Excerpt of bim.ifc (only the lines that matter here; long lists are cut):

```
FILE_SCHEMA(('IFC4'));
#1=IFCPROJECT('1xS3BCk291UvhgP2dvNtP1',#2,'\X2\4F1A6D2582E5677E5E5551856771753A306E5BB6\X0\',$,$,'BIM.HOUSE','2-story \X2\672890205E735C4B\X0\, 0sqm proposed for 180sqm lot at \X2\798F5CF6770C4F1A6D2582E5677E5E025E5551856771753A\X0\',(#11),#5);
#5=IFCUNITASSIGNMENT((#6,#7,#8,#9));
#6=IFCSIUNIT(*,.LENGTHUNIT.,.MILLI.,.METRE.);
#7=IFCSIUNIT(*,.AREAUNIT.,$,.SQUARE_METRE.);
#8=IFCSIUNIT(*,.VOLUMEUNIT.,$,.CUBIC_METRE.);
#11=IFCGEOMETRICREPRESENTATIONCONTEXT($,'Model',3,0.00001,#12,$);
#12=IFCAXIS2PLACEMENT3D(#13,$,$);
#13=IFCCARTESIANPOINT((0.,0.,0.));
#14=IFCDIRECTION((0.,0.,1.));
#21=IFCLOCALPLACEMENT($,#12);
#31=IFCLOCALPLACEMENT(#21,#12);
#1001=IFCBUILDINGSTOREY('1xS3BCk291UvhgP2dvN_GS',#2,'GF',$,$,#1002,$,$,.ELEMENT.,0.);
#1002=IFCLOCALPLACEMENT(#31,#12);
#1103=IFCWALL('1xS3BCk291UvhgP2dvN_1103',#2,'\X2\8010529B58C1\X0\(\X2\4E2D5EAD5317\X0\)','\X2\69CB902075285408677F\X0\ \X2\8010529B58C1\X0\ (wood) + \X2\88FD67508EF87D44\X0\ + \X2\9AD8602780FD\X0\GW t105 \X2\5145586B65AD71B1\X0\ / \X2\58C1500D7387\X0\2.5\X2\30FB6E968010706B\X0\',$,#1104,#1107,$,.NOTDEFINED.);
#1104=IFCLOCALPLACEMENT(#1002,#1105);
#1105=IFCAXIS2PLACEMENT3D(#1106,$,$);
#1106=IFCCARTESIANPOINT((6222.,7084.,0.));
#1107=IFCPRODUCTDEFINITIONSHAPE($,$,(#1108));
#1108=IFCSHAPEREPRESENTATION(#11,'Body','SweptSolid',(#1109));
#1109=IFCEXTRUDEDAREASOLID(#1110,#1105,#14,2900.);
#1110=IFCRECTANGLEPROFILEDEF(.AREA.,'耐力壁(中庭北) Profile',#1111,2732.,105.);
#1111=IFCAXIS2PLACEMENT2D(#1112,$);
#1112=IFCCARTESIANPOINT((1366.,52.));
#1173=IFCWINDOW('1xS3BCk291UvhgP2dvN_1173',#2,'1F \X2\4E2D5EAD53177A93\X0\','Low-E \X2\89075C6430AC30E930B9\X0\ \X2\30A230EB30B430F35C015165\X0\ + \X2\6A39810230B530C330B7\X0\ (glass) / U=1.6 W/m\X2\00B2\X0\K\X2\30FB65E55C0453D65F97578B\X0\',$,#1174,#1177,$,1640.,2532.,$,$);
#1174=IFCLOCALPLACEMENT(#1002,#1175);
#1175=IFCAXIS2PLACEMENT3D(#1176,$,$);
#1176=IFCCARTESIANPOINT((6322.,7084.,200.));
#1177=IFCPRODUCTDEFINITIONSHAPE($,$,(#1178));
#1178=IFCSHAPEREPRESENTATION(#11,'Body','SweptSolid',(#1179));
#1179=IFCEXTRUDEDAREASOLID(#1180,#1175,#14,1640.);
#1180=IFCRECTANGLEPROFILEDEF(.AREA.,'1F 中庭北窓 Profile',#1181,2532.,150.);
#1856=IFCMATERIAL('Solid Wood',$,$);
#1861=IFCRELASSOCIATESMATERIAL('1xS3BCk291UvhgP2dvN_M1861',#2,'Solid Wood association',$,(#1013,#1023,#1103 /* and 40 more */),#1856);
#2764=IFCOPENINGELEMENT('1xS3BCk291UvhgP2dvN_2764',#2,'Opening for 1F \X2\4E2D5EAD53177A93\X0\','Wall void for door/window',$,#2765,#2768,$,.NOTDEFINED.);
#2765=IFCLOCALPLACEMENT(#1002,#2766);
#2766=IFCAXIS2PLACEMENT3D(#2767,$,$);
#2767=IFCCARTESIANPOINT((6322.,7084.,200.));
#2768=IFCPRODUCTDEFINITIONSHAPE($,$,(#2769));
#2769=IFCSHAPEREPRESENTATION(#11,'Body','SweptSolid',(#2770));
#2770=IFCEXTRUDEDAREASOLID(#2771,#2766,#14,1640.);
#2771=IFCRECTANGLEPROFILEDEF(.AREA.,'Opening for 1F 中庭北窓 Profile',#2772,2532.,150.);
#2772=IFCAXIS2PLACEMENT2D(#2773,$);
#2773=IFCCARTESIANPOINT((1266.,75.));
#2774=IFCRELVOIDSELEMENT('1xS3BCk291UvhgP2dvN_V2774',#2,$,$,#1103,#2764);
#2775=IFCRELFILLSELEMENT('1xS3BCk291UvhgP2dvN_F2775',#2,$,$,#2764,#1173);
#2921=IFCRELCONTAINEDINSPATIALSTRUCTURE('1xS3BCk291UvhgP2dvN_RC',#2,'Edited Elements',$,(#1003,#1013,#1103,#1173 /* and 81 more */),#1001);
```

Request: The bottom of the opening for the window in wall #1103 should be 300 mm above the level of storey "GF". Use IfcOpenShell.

```python
import numpy as np
import ifcopenshell
import ifcopenshell.api.geometry
import ifcopenshell.geom
import ifcopenshell.util.element
import ifcopenshell.util.placement
import ifcopenshell.util.shape
import ifcopenshell.util.unit

model = ifcopenshell.open("bim.ifc")
unit_scale = ifcopenshell.util.unit.calculate_unit_scale(model)

window = model.by_guid("1xS3BCk291UvhgP2dvN_1173")
opening = window.FillsVoids[0].RelatingOpeningElement
storey = ifcopenshell.util.element.get_container(window, ifc_class="IfcBuildingStorey")
level = ifcopenshell.util.placement.get_local_placement(storey.ObjectPlacement)[2, 3]

# The opening's origin need not be at the sill, so measure its lowest point.
shape = ifcopenshell.geom.create_shape(ifcopenshell.geom.settings(), opening)
bottom = ifcopenshell.util.shape.get_shape_bottom_elevation(shape, shape.geometry) / unit_scale
dz = level + 300.0 - bottom

shift = np.array([0.0, 0.0, dz])
# The window is not placed relative to its opening, so move both.
for product in (opening, window):
    matrix = ifcopenshell.util.placement.get_local_placement(product.ObjectPlacement)
    matrix[:3, 3] += shift
    ifcopenshell.api.geometry.edit_object_placement(model, product=product, matrix=matrix, is_si=False)

print(f"moved by {dz * unit_scale:+.3f} m")

model.write("bim_v2.ifc")
```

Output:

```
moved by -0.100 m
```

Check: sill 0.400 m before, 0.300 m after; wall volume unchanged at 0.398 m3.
